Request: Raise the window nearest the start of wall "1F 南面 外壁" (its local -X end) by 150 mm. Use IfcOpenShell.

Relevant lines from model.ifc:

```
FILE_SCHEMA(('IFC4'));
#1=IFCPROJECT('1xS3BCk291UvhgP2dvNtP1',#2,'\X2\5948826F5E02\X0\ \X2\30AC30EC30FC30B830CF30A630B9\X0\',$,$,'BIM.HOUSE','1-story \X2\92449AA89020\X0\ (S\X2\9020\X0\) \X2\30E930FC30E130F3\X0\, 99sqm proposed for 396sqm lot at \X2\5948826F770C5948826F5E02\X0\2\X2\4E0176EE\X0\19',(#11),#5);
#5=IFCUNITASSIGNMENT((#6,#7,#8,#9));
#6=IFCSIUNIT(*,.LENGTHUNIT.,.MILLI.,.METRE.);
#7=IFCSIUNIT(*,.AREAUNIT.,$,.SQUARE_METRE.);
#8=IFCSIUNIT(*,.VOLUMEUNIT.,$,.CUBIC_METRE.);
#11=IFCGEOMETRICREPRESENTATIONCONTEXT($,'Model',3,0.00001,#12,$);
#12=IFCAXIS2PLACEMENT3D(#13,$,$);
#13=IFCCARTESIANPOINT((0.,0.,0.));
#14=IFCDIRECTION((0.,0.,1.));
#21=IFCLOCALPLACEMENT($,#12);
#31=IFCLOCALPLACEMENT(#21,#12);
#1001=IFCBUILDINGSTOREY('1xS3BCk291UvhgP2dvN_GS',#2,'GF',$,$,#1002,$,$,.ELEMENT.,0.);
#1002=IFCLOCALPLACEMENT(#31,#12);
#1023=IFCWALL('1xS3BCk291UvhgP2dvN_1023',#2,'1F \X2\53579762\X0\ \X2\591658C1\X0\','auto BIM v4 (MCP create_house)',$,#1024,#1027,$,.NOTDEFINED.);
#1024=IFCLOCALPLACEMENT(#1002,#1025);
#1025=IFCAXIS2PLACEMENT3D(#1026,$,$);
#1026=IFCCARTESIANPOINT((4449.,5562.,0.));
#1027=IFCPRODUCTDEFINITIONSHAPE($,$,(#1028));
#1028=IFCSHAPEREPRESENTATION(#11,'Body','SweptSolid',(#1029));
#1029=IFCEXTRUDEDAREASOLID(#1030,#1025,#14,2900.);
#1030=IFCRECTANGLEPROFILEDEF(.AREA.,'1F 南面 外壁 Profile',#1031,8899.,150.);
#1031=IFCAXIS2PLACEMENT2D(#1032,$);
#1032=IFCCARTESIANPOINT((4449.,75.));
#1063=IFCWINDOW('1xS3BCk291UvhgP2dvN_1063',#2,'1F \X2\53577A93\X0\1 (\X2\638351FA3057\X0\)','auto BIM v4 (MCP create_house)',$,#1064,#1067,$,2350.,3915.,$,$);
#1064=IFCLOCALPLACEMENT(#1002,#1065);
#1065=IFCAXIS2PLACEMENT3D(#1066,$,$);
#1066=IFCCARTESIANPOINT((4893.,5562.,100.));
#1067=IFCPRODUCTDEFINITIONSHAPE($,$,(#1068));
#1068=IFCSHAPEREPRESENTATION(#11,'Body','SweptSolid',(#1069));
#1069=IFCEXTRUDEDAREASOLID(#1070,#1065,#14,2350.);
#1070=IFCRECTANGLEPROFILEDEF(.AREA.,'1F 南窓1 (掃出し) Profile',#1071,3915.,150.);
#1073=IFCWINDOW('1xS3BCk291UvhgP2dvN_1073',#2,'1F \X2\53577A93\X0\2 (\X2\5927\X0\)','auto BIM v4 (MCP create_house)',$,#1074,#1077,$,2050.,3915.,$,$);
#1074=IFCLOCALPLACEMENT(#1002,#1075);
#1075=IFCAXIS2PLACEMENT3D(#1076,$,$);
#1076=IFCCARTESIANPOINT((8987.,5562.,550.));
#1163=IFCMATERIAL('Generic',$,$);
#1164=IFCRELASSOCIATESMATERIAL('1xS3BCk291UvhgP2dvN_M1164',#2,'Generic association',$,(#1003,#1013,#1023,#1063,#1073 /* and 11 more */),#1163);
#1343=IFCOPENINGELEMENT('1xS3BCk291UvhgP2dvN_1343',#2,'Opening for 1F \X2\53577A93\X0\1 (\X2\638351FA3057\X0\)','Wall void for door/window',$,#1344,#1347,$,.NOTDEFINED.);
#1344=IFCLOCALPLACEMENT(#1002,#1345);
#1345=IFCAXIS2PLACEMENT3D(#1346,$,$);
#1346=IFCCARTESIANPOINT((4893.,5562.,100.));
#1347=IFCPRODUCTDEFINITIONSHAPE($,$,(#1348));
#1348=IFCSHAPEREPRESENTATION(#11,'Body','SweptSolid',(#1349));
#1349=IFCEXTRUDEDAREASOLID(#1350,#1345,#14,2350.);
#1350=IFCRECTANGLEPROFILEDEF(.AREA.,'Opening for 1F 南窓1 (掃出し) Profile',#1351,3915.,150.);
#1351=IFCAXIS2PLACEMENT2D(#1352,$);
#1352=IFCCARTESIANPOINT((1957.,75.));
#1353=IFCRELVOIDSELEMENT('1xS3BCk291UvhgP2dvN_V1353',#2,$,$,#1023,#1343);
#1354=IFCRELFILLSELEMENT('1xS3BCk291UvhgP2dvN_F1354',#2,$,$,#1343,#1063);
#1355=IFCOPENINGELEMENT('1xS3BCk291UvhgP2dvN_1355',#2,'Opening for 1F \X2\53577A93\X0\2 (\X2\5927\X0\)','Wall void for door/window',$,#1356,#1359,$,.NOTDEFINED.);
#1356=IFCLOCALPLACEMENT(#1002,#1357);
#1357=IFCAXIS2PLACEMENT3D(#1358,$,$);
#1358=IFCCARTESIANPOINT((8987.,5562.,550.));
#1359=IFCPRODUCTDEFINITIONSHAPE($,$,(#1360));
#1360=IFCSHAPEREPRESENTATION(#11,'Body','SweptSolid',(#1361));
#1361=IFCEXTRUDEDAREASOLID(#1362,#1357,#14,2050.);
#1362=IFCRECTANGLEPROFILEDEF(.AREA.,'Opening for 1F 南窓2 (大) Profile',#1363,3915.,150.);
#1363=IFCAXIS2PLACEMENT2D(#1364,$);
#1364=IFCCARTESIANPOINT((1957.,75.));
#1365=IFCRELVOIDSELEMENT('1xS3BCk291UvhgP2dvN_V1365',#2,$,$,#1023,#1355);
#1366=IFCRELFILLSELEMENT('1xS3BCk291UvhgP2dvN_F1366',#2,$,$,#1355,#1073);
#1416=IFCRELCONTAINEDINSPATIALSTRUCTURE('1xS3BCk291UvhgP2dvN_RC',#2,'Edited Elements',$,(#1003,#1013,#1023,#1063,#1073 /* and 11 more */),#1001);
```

```python
import numpy as np
import ifcopenshell
import ifcopenshell.api.geometry
import ifcopenshell.util.placement
import ifcopenshell.util.unit

model = ifcopenshell.open("model.ifc")
unit_scale = ifcopenshell.util.unit.calculate_unit_scale(model)

window = model.by_guid("1xS3BCk291UvhgP2dvN_1063")
opening = window.FillsVoids[0].RelatingOpeningElement
dz = 150.0

shift = np.array([0.0, 0.0, dz])
# The window is not placed relative to its opening, so move both.
for product in (opening, window):
    matrix = ifcopenshell.util.placement.get_local_placement(product.ObjectPlacement)
    matrix[:3, 3] += shift
    ifcopenshell.api.geometry.edit_object_placement(model, product=product, matrix=matrix, is_si=False)

print(f"moved by {dz * unit_scale:+.3f} m")

model.write("model_updated.ifc")
```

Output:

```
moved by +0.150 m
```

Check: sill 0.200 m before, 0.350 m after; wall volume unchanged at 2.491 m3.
